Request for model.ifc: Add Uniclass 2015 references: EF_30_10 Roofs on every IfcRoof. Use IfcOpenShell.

First a look at what the model holds.

```python
import ifcopenshell

model = ifcopenshell.open("model.ifc")
print(model.schema)
print("classifications:", [c.Name for c in model.by_type("IfcClassification")])
for ifc_class in ("IfcDoor", "IfcRoof", "IfcStair", "IfcWall", "IfcWindow"):
    print(ifc_class, len(model.by_type(ifc_class)))
```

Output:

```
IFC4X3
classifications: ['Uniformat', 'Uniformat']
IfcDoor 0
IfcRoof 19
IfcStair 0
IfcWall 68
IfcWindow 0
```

```python
import ifcopenshell
import ifcopenshell.api.classification

model = ifcopenshell.open("model.ifc")

system = ifcopenshell.api.classification.add_classification(model, classification="Uniclass 2015")

codes = {
    "IfcRoof": ("EF_30_10", "Roofs"),
}
for ifc_class, (code, name) in codes.items():
    products = model.by_type(ifc_class)
    ifcopenshell.api.classification.add_reference(
        model, products=products, classification=system, identification=code, name=name
    )
    print(code, len(products))

model.write("model_rev.ifc")
```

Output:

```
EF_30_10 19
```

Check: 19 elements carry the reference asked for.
